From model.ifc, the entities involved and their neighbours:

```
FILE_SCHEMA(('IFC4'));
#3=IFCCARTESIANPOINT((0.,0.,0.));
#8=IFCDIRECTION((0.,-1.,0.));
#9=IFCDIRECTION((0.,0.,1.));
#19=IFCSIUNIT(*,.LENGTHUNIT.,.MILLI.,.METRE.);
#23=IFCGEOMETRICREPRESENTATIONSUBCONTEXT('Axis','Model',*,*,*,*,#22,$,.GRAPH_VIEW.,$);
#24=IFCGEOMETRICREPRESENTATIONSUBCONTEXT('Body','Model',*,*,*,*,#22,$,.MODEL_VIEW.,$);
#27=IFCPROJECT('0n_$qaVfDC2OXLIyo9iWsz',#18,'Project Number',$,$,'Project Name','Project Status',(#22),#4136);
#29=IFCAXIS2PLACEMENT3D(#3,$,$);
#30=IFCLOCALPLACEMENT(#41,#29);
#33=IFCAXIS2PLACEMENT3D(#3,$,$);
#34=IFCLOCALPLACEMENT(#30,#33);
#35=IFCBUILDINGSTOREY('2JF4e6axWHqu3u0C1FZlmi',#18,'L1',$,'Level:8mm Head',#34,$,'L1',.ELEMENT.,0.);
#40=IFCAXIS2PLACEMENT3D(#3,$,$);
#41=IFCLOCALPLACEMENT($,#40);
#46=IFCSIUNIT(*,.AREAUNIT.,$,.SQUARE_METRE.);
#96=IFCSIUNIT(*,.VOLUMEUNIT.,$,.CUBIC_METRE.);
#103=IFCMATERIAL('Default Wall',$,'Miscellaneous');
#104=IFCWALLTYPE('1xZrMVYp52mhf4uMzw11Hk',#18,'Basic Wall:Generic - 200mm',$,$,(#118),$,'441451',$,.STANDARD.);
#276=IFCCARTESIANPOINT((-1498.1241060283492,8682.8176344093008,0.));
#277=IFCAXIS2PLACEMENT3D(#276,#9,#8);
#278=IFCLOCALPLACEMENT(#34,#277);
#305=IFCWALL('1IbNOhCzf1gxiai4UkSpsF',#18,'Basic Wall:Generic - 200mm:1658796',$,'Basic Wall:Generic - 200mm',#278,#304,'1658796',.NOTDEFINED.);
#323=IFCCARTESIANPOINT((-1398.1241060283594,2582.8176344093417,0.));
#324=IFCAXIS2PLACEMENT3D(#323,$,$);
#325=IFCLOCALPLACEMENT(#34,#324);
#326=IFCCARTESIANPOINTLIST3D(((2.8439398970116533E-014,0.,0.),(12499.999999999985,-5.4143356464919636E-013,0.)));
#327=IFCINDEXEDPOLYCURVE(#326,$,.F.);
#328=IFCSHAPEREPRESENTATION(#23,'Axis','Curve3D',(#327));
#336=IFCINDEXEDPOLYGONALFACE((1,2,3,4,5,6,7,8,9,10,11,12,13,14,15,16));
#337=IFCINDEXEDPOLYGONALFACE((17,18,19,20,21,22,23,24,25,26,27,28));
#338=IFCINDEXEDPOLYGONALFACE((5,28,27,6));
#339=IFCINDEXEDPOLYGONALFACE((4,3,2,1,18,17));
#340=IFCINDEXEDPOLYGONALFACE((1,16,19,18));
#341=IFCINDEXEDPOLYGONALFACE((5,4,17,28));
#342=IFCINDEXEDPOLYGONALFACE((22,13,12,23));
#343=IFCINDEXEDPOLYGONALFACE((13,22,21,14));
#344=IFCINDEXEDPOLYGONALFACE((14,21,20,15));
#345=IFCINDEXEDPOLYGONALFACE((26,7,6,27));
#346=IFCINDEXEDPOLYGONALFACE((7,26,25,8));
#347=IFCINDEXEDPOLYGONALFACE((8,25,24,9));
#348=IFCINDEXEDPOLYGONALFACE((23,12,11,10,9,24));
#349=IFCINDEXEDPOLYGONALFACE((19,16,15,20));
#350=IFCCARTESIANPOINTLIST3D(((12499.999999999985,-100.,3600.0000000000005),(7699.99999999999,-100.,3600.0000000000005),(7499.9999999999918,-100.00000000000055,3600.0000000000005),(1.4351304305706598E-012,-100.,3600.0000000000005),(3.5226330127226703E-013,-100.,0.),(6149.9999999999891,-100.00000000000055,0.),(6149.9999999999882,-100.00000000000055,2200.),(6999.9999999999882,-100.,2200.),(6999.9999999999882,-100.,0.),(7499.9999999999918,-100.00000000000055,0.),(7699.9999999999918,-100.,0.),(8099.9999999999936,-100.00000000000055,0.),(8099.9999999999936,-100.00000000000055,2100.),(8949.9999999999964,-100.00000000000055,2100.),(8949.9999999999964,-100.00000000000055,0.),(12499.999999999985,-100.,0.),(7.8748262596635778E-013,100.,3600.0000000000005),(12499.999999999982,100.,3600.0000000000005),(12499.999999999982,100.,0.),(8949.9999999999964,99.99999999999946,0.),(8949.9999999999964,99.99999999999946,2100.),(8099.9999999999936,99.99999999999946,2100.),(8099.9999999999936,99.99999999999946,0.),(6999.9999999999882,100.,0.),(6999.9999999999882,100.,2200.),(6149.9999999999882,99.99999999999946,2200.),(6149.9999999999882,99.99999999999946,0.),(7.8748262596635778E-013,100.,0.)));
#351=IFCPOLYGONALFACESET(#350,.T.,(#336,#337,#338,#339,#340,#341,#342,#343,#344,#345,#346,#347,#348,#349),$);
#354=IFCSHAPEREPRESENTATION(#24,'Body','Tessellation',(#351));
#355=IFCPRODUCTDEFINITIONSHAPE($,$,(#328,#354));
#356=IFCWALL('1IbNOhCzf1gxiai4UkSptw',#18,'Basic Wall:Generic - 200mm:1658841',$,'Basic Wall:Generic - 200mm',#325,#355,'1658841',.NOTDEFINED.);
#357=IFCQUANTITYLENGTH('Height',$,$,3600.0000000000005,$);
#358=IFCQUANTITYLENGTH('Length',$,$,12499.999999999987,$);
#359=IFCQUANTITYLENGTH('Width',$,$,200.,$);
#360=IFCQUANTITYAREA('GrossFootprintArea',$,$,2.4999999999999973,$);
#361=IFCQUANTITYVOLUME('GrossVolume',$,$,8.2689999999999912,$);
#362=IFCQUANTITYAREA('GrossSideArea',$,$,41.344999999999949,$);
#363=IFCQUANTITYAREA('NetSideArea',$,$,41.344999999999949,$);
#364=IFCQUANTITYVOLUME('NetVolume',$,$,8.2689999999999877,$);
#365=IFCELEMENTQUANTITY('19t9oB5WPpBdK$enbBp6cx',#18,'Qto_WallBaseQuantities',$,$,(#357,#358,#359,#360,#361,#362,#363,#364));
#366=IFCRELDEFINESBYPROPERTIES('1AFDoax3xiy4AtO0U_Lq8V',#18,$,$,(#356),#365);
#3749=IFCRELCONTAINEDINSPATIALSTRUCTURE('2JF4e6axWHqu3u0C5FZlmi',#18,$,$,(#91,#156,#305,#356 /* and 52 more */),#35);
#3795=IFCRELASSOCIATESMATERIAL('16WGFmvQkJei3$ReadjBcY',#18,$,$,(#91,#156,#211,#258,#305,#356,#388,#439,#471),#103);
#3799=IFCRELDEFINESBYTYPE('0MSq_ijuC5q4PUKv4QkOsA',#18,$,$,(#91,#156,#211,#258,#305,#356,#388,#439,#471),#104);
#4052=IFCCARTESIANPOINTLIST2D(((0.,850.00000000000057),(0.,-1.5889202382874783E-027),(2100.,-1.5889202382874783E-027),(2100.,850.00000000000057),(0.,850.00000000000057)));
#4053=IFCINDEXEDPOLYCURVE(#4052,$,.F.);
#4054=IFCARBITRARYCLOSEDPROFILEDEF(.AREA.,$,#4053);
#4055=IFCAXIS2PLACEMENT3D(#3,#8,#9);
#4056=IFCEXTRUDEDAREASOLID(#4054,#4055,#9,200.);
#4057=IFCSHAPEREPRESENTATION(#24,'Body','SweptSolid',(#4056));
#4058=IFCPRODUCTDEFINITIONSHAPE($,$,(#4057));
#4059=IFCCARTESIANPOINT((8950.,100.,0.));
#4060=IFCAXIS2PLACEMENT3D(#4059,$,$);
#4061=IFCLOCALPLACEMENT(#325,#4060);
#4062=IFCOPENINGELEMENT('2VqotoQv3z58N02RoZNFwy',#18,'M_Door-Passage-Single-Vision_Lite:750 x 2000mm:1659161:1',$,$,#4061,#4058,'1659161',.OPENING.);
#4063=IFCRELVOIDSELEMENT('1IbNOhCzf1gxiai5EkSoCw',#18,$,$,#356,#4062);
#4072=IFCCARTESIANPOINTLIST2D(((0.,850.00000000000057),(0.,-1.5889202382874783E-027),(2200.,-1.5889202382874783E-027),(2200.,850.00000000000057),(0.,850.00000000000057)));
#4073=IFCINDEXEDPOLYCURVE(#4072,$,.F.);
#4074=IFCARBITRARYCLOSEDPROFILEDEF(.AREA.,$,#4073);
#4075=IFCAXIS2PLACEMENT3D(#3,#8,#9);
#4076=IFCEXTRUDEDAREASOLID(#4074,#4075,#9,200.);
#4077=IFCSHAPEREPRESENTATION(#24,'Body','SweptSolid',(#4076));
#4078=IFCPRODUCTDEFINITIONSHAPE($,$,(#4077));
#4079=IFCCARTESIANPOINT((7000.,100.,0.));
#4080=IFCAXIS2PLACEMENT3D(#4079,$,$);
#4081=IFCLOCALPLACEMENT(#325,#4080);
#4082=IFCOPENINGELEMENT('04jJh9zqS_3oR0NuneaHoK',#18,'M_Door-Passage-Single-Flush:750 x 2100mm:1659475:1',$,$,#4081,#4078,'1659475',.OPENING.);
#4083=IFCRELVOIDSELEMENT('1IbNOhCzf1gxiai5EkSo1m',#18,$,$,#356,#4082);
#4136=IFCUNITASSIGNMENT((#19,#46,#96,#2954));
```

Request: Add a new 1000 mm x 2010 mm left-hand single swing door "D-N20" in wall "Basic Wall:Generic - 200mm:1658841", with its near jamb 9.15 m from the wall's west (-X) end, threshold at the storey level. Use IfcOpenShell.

```python
import numpy as np
import ifcopenshell
import ifcopenshell.api.feature
import ifcopenshell.api.geometry
import ifcopenshell.api.pset
import ifcopenshell.api.root
import ifcopenshell.api.spatial
import ifcopenshell.geom
import ifcopenshell.util.element
import ifcopenshell.util.placement
import ifcopenshell.util.representation
import ifcopenshell.util.shape
import ifcopenshell.util.unit

model = ifcopenshell.open("model.ifc")
unit_scale = ifcopenshell.util.unit.calculate_unit_scale(model)
area_scale = ifcopenshell.util.unit.calculate_unit_scale(model, "AREAUNIT")
volume_scale = ifcopenshell.util.unit.calculate_unit_scale(model, "VOLUMEUNIT")
settings = ifcopenshell.geom.settings()


def volume(element):
    """Net volume in cubic metres, openings subtracted."""
    shape = ifcopenshell.geom.create_shape(settings, element)
    return ifcopenshell.util.shape.get_volume(shape.geometry)


wall = model.by_id(356)
storey = ifcopenshell.util.element.get_container(wall, ifc_class="IfcBuildingStorey")
context = ifcopenshell.util.representation.get_context(model, "Model", "Body", "MODEL_VIEW")
before = volume(wall)

width, height, from_end, sill = 1, 2.01, 9.15, 0.0  # metres

# The wall runs along its own X axis, and the end named is its -X end.
wall_shape = ifcopenshell.geom.create_shape(settings, wall)
x, y, z = ifcopenshell.util.shape.get_vertices(wall_shape.geometry).T
start = x.min() + from_end
face, thickness = float(y.min()), float(y.max() - y.min())
wall_matrix = ifcopenshell.util.placement.get_local_placement(wall.ObjectPlacement)
level = ifcopenshell.util.placement.get_local_placement(storey.ObjectPlacement)[2, 3]


def in_wall(x, y):
    """Placement at x, y metres in the wall's axes, at sill height."""
    matrix = wall_matrix.copy()
    matrix[:, 3] = wall_matrix @ np.array([x / unit_scale, y / unit_scale, 0.0, 1.0])
    matrix[2, 3] = level + sill / unit_scale
    return matrix


# Opening: a box that overshoots both wall faces by 50 mm.
opening = ifcopenshell.api.root.create_entity(model, ifc_class="IfcOpeningElement", predefined_type="OPENING")
box = ifcopenshell.api.geometry.add_wall_representation(
    model, context=context, length=width, height=height, thickness=thickness + 0.1
)
ifcopenshell.api.geometry.assign_representation(model, product=opening, representation=box)
ifcopenshell.api.geometry.edit_object_placement(model, product=opening, matrix=in_wall(start, face - 0.05), is_si=False)
ifcopenshell.api.feature.add_feature(model, feature=opening, element=wall)

door = ifcopenshell.api.root.create_entity(model, ifc_class="IfcDoor", name="D-N20", predefined_type="DOOR")
door.OverallWidth, door.OverallHeight = width / unit_scale, height / unit_scale
door.OperationType = "SINGLE_SWING_LEFT"
body = ifcopenshell.api.geometry.add_door_representation(
    model,
    context=context,
    overall_width=door.OverallWidth,
    overall_height=door.OverallHeight,
    operation_type="SINGLE_SWING_LEFT",
    lining_properties={"LiningDepth": thickness / unit_scale, "ThresholdDepth": thickness / unit_scale},
)
ifcopenshell.api.geometry.assign_representation(model, product=door, representation=body)
ifcopenshell.api.spatial.assign_container(model, products=[door], relating_structure=storey)
ifcopenshell.api.feature.add_filling(model, opening=opening, element=door)

# The lining spans the wall, so the door starts at the wall face.
ifcopenshell.api.geometry.edit_object_placement(model, product=door, matrix=in_wall(start, face), is_si=False)

after = volume(wall)

# Update the wall's stored quantities.
qto = model.by_id(ifcopenshell.util.element.get_pset(wall, "Qto_WallBaseQuantities", should_inherit=False)["id"])
ifcopenshell.api.pset.edit_qto(model, qto=qto, properties={
    "NetSideArea": after / thickness / area_scale,
    "NetVolume": after / volume_scale,
})

print(f"wall volume {before:.3f} -> {after:.3f} m3")

model.write("model_v2.ifc")
```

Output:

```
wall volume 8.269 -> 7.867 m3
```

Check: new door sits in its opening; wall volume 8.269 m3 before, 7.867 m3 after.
